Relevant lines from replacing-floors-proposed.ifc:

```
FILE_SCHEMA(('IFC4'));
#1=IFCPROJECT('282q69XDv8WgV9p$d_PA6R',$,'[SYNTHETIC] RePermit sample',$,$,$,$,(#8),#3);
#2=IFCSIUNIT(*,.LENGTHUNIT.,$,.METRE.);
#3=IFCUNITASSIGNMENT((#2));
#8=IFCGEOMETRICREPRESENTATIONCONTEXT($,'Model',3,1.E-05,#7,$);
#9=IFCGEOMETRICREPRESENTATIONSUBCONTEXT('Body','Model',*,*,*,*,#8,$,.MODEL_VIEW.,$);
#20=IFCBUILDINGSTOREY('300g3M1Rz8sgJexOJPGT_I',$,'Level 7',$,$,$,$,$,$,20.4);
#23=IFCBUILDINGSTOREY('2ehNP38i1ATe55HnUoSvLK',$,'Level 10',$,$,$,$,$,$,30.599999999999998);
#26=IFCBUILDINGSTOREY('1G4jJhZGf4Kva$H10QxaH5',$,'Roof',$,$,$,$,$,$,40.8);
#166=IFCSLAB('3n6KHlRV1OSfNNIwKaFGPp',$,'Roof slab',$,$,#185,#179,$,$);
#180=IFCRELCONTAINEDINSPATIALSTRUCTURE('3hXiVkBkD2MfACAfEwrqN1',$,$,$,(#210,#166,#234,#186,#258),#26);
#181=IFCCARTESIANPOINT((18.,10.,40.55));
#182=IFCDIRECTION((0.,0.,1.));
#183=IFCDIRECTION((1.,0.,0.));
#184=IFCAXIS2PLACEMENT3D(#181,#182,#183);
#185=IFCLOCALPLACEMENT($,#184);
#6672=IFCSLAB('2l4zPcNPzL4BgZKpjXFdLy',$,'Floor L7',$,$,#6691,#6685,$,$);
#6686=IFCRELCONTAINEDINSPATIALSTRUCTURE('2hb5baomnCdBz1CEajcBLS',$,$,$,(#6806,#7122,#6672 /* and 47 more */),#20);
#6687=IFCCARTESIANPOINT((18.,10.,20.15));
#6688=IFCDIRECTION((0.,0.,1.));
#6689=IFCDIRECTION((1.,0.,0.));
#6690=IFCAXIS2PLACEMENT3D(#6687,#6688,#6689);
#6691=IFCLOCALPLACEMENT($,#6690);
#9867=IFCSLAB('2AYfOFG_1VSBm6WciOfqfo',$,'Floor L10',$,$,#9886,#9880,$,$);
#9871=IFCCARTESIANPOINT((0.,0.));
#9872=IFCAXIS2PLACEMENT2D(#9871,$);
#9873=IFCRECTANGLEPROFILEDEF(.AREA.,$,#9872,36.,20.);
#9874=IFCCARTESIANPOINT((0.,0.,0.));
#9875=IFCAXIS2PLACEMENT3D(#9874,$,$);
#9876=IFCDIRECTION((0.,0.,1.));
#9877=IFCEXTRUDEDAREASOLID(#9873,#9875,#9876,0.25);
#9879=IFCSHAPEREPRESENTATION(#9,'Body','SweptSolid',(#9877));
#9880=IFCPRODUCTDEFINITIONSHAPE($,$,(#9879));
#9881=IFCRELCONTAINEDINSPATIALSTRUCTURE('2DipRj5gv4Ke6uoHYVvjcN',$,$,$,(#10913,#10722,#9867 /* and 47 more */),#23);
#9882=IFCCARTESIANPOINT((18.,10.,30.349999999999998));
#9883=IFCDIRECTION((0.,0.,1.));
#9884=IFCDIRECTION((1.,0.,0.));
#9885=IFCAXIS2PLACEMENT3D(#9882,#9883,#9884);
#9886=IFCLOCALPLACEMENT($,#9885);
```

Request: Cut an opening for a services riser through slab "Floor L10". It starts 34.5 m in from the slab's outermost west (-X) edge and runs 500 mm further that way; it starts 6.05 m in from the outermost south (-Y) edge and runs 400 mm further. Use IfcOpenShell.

```python
import numpy as np
import ifcopenshell
import ifcopenshell.api.feature
import ifcopenshell.api.geometry
import ifcopenshell.api.root
import ifcopenshell.geom
import ifcopenshell.util.placement
import ifcopenshell.util.representation
import ifcopenshell.util.shape
import ifcopenshell.util.unit

model = ifcopenshell.open("replacing-floors-proposed.ifc")
unit_scale = ifcopenshell.util.unit.calculate_unit_scale(model)
settings = ifcopenshell.geom.settings()


def volume(element):
    """Net volume in cubic metres, openings subtracted."""
    shape = ifcopenshell.geom.create_shape(settings, element)
    return ifcopenshell.util.shape.get_volume(shape.geometry)


slab = model.by_id(9867)
before = volume(slab)

# Extent in the slab's own axes, in metres. The edges named are its -X and -Y sides.
slab_shape = ifcopenshell.geom.create_shape(settings, slab)
vertices = ifcopenshell.util.shape.get_vertices(slab_shape.geometry)
x_min, y_min, bottom = vertices.min(axis=0)
top = vertices[:, 2].max()

opening = ifcopenshell.api.root.create_entity(model, ifc_class="IfcOpeningElement", name="Services riser opening", predefined_type="OPENING")
context = ifcopenshell.util.representation.get_context(model, "Model", "Body", "MODEL_VIEW")
width, depth = 0.5, 0.4
outline = [(0.0, 0.0), (width, 0.0), (width, depth), (0.0, depth), (0.0, 0.0)]
# Overshoot both faces by 50 mm so the cut is clean.
shape = ifcopenshell.api.geometry.add_slab_representation(
    model, context=context, depth=top - bottom + 0.1, polyline=outline
)
ifcopenshell.api.geometry.assign_representation(model, product=opening, representation=shape)

matrix = ifcopenshell.util.placement.get_local_placement(slab.ObjectPlacement)
matrix[:, 3] = matrix @ np.append(np.array([x_min + 34.5, y_min + 6.05, bottom - 0.05]) / unit_scale, 1.0)
ifcopenshell.api.geometry.edit_object_placement(model, product=opening, matrix=matrix, is_si=False)
ifcopenshell.api.feature.add_feature(model, feature=opening, element=slab)

after = volume(slab)

print(f"slab volume {before:.3f} -> {after:.3f} m3")

model.write("replacing-floors-proposed-out.ifc")
```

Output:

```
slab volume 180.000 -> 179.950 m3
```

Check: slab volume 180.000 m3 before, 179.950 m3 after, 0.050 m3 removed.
